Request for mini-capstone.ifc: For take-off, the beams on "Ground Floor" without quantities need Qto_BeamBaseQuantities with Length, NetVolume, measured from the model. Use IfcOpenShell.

First a look at what the model holds.

```python
import ifcopenshell
import ifcopenshell.util.element
import ifcopenshell.util.unit

model = ifcopenshell.open("mini-capstone.ifc")
print(model.schema)
for unit_type in ("LENGTHUNIT", "AREAUNIT", "VOLUMEUNIT"):
    print(unit_type, ifcopenshell.util.unit.calculate_unit_scale(model, unit_type))
storey = next(s for s in model.by_type("IfcBuildingStorey") if s.Name == "Ground Floor")
beams = [e for e in ifcopenshell.util.element.get_decomposition(storey) if e.is_a("IfcBeam")]
for e in sorted(beams, key=lambda e: e.id()):
    print(e.id(), e.is_a(), e.Name, list(ifcopenshell.util.element.get_psets(e, qtos_only=True)), sep=" | ")
```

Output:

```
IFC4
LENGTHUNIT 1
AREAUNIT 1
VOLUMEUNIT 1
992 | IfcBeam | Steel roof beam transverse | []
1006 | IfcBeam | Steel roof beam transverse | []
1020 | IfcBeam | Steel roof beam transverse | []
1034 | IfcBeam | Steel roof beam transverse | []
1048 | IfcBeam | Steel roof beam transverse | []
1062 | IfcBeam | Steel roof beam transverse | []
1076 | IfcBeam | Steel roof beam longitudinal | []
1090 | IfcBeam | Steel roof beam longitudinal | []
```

```python
import ifcopenshell
import ifcopenshell.api.pset
import ifcopenshell.geom
import ifcopenshell.util.element
import ifcopenshell.util.shape
import ifcopenshell.util.unit

model = ifcopenshell.open("mini-capstone.ifc")
unit_scale = ifcopenshell.util.unit.calculate_unit_scale(model)
volume_scale = ifcopenshell.util.unit.calculate_unit_scale(model, "VOLUMEUNIT")
settings = ifcopenshell.geom.settings()

storey = next(s for s in model.by_type("IfcBuildingStorey") if s.Name == "Ground Floor")
beams = [e for e in ifcopenshell.util.element.get_decomposition(storey) if e.is_a("IfcBeam")]

for e in sorted(beams, key=lambda e: e.id()):
    if ifcopenshell.util.element.get_psets(e, qtos_only=True, should_inherit=False):
        continue
    # Geometry comes back in metres, in the element's own axes.
    shape = ifcopenshell.geom.create_shape(settings, e)
    values = {
        "Length": ifcopenshell.util.shape.get_max_xyz(shape.geometry) / unit_scale,
        "NetVolume": ifcopenshell.util.shape.get_volume(shape.geometry) / volume_scale,
    }
    qto = ifcopenshell.api.pset.add_qto(model, product=e, name="Qto_BeamBaseQuantities")
    ifcopenshell.api.pset.edit_qto(model, qto=qto, properties=values)
    print(e.id(), {k: round(v, 3) for k, v in values.items()})

model.write("mini-capstone-out.ifc")
```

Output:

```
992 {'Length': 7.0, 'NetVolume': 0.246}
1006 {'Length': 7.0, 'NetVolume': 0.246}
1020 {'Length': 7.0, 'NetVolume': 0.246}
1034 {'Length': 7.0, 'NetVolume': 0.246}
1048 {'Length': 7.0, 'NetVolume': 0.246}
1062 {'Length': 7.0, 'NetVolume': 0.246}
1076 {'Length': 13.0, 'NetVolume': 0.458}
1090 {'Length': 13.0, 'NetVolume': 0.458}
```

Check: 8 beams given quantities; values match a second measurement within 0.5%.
